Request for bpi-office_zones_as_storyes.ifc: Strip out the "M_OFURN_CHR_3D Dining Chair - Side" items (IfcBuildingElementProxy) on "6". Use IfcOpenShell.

First a look at what the model holds.

```python
import ifcopenshell
import ifcopenshell.util.element

model = ifcopenshell.open("bpi-office_zones_as_storyes.ifc")
print(model.schema)
storey = next(s for s in model.by_type("IfcBuildingStorey") if s.Name == "6")
proxies = [e for e in ifcopenshell.util.element.get_decomposition(storey) if e.is_a("IfcBuildingElementProxy")]
seen = {}
for e in proxies:
    element_type = ifcopenshell.util.element.get_type(e)
    name = element_type.Name if element_type not in (None, e) else None
    seen[name] = seen.get(name, 0) + 1
for name, count in sorted(seen.items(), key=str):
    print(count, "x", name)
```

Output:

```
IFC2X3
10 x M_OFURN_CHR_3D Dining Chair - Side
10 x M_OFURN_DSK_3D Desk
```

```python
import ifcopenshell
import ifcopenshell.api.root
import ifcopenshell.util.element

model = ifcopenshell.open("bpi-office_zones_as_storyes.ifc")

storey = next(s for s in model.by_type("IfcBuildingStorey") if s.Name == "6")
proxies = [e for e in ifcopenshell.util.element.get_decomposition(storey) if e.is_a("IfcBuildingElementProxy")]
targets = [e for e in proxies if (t := ifcopenshell.util.element.get_type(e)) not in (None, e) and t.Name == "M_OFURN_CHR_3D Dining Chair - Side"]

for e in targets:
    ifcopenshell.api.root.remove_product(model, product=e)
print(len(targets), "removed")

model.write("bpi-office_zones_as_storyes_v2.ifc")
```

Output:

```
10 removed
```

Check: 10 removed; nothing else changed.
